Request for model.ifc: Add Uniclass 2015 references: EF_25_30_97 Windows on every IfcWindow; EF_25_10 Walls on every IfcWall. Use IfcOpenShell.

First a look at what the model holds.

```python
import ifcopenshell

model = ifcopenshell.open("model.ifc")
print(model.schema)
print("classifications:", [c.Name for c in model.by_type("IfcClassification")])
for ifc_class in ("IfcDoor", "IfcRoof", "IfcStair", "IfcWall", "IfcWindow"):
    print(ifc_class, len(model.by_type(ifc_class)))
```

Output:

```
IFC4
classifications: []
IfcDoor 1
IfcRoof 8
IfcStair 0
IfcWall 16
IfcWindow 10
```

```python
import ifcopenshell
import ifcopenshell.api.classification

model = ifcopenshell.open("model.ifc")

system = ifcopenshell.api.classification.add_classification(model, classification="Uniclass 2015")

codes = {
    "IfcWindow": ("EF_25_30_97", "Windows"),
    "IfcWall": ("EF_25_10", "Walls"),
}
for ifc_class, (code, name) in codes.items():
    products = model.by_type(ifc_class)
    ifcopenshell.api.classification.add_reference(
        model, products=products, classification=system, identification=code, name=name
    )
    print(code, len(products))

model.write("model_v2.ifc")
```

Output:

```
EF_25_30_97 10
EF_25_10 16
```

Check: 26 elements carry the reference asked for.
